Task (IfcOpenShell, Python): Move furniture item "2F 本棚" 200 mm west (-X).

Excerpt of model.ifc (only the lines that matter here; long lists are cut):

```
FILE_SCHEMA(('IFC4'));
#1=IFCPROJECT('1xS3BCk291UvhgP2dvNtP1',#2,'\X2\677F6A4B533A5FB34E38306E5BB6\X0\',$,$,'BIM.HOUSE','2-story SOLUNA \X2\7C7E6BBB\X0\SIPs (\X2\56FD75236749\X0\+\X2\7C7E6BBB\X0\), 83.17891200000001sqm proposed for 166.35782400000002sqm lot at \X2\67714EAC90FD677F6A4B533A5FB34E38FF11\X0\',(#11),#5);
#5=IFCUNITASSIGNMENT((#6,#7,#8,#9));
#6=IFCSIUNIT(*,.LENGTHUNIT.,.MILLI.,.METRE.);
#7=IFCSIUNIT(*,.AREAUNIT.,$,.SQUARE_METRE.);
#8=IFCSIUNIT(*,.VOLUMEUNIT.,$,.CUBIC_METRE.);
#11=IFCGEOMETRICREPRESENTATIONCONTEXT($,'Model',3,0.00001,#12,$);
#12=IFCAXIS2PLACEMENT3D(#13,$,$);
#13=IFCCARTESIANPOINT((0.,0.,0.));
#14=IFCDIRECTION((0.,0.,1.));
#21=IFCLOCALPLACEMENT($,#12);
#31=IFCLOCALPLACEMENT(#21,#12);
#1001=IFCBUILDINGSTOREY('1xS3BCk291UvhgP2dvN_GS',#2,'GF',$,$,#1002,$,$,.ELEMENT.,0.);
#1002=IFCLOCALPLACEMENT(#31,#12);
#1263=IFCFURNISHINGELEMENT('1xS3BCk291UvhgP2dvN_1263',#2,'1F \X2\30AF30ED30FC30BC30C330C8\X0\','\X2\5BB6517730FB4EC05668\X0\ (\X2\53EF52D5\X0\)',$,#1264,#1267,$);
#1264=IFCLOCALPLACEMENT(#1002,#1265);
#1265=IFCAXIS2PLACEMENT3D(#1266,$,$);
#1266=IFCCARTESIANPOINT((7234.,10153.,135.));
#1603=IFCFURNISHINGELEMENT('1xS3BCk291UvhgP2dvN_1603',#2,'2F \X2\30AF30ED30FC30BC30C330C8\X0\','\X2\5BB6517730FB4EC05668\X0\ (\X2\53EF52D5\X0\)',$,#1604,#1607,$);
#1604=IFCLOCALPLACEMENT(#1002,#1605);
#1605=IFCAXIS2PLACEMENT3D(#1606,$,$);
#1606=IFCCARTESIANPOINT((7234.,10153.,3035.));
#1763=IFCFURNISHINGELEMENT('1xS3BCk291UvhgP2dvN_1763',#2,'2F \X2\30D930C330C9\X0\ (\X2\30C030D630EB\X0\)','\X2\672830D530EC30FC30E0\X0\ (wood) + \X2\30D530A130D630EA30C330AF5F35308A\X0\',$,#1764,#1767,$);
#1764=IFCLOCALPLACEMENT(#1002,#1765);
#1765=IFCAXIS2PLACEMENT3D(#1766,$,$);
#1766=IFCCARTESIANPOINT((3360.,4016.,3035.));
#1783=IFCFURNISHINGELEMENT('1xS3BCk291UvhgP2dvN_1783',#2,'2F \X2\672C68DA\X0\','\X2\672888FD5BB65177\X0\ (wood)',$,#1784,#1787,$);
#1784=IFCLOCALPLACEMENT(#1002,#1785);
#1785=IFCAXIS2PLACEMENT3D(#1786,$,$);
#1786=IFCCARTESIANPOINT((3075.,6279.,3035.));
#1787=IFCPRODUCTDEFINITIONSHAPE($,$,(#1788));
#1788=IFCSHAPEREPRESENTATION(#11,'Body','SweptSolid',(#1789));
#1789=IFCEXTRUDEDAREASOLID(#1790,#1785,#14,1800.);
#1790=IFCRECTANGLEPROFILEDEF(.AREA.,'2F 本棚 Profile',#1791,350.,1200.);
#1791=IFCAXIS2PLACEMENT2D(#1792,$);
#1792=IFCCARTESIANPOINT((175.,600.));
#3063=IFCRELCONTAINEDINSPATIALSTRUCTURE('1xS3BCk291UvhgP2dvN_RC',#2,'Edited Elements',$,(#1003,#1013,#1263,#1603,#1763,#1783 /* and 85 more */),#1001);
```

```python
import ifcopenshell
import ifcopenshell.api.geometry
import ifcopenshell.util.placement
import ifcopenshell.util.unit

model = ifcopenshell.open("model.ifc")
unit_scale = ifcopenshell.util.unit.calculate_unit_scale(model)

item = model.by_id(1783)
matrix = ifcopenshell.util.placement.get_local_placement(item.ObjectPlacement)
matrix[0, 3] -= 0.2 / unit_scale
ifcopenshell.api.geometry.edit_object_placement(model, product=item, matrix=matrix, is_si=False)

print(ifcopenshell.util.placement.get_local_placement(item.ObjectPlacement).round(3) + 0.0)

model.write("model_updated.ifc")
```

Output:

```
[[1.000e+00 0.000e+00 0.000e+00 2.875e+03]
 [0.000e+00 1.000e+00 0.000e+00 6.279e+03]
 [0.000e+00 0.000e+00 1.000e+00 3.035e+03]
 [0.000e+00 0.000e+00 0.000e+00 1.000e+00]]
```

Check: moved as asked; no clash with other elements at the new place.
